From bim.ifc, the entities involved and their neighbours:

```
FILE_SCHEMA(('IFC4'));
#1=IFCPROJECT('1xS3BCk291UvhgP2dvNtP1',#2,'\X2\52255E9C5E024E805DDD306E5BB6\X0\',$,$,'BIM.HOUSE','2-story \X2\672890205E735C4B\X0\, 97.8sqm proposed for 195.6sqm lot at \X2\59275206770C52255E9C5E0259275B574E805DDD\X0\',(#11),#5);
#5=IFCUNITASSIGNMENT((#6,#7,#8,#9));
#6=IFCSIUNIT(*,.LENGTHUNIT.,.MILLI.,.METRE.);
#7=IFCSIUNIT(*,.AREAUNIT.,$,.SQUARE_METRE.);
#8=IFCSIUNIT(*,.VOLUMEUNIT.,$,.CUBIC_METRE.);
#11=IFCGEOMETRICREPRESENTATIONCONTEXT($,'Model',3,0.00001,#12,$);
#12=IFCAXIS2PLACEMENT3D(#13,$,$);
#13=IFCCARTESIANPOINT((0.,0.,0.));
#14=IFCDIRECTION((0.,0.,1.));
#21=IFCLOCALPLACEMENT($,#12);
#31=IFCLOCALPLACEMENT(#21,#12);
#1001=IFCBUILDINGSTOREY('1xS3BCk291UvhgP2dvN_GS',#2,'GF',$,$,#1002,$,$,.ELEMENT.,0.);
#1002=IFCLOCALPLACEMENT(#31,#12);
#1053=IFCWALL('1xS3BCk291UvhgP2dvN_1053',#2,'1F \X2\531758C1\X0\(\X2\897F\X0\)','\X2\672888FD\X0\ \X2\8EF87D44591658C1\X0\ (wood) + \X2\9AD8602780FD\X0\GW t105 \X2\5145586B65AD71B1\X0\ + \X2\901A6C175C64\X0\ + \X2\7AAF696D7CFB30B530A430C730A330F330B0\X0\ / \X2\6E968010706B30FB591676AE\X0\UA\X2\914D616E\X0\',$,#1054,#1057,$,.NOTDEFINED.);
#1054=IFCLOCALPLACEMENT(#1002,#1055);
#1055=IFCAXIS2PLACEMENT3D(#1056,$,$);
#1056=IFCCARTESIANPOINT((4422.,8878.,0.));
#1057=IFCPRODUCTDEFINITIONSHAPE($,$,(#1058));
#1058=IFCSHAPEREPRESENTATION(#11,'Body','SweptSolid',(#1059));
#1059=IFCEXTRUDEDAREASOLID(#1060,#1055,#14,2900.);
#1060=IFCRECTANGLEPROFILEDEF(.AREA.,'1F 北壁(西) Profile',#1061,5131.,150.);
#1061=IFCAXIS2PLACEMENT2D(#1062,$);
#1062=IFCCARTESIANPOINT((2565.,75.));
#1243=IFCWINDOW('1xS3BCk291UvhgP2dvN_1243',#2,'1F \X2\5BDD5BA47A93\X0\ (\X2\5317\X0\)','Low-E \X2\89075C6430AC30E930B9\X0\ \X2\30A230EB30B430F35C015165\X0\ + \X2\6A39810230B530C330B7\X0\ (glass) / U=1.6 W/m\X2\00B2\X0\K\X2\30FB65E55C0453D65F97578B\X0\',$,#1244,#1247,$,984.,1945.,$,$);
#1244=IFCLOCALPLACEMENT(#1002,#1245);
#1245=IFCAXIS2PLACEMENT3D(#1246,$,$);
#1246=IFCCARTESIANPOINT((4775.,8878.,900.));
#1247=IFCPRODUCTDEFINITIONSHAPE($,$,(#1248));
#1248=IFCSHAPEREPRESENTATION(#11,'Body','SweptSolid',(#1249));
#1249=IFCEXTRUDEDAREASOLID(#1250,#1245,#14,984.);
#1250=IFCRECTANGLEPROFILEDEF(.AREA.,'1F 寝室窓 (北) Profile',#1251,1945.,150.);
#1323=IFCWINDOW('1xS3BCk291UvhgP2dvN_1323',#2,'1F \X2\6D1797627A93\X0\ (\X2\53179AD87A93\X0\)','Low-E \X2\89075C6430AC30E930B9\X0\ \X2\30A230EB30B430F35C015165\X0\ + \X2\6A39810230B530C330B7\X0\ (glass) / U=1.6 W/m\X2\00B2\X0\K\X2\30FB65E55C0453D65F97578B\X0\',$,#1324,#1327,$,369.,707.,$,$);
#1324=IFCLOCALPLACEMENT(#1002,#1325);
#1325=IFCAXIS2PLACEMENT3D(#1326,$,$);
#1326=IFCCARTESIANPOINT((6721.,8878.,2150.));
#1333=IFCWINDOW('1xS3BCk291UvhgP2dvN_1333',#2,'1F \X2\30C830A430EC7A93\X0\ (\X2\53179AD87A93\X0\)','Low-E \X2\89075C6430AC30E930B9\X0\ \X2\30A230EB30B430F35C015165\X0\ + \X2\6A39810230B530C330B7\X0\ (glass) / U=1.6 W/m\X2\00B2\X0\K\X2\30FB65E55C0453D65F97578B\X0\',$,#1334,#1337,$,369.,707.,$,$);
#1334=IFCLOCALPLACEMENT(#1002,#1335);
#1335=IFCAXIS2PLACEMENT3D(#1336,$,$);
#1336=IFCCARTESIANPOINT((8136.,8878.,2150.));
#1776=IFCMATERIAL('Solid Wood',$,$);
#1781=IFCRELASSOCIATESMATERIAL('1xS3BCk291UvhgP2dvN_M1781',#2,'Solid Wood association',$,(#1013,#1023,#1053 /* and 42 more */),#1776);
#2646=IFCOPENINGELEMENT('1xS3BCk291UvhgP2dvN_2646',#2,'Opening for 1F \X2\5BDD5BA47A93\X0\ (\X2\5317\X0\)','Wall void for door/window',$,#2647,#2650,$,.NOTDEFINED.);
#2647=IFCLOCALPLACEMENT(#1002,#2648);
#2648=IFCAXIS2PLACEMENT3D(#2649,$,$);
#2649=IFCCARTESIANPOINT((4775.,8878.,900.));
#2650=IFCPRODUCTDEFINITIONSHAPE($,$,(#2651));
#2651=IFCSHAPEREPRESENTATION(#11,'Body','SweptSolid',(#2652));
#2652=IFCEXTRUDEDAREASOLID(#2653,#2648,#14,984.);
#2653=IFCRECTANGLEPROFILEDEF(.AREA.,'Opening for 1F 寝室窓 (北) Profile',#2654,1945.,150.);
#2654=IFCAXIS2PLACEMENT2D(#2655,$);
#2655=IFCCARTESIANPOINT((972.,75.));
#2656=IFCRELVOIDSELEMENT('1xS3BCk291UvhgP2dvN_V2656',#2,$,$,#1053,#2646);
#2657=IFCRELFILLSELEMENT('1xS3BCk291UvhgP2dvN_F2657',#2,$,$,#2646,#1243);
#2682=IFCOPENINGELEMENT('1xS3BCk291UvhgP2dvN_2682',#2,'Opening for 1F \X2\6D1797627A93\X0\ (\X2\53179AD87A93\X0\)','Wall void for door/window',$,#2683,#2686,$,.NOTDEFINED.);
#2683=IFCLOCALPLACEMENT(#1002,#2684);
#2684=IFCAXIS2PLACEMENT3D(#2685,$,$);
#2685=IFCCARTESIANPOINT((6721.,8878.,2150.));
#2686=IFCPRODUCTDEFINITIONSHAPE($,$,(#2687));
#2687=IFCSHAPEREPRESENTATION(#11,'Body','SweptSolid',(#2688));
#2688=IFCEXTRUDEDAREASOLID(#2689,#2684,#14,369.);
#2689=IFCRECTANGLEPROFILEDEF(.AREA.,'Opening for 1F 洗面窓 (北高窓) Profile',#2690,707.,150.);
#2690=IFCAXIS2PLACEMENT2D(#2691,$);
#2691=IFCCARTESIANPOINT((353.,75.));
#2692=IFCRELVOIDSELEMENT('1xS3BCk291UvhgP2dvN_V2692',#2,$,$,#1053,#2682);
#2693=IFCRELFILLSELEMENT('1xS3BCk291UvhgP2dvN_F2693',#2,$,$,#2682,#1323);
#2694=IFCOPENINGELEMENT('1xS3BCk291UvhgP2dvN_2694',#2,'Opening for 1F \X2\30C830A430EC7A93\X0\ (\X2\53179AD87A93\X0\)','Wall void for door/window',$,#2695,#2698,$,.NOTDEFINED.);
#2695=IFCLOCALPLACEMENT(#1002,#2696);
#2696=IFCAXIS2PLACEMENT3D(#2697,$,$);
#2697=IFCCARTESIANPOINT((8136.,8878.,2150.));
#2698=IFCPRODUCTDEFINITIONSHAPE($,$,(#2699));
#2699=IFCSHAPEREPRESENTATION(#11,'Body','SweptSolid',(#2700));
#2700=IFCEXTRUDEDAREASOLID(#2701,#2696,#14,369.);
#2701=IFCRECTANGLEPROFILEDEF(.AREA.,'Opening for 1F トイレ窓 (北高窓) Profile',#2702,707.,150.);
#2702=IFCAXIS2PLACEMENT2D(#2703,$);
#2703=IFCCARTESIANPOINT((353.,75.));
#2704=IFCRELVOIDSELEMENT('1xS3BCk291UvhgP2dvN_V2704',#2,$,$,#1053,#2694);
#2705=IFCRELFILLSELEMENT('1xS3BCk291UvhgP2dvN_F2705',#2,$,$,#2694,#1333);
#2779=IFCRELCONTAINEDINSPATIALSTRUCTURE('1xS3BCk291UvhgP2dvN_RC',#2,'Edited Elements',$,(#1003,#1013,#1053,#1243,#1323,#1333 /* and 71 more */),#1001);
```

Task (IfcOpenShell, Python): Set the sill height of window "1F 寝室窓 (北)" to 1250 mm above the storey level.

```python
import numpy as np
import ifcopenshell
import ifcopenshell.api.geometry
import ifcopenshell.geom
import ifcopenshell.util.element
import ifcopenshell.util.placement
import ifcopenshell.util.shape
import ifcopenshell.util.unit

model = ifcopenshell.open("bim.ifc")
unit_scale = ifcopenshell.util.unit.calculate_unit_scale(model)

window = model.by_guid("1xS3BCk291UvhgP2dvN_1243")
opening = window.FillsVoids[0].RelatingOpeningElement
storey = ifcopenshell.util.element.get_container(window, ifc_class="IfcBuildingStorey")
level = ifcopenshell.util.placement.get_local_placement(storey.ObjectPlacement)[2, 3]

# The opening's origin need not be at the sill, so measure its lowest point.
shape = ifcopenshell.geom.create_shape(ifcopenshell.geom.settings(), opening)
bottom = ifcopenshell.util.shape.get_shape_bottom_elevation(shape, shape.geometry) / unit_scale
dz = level + 1250.0 - bottom

shift = np.array([0.0, 0.0, dz])
# The window is not placed relative to its opening, so move both.
for product in (opening, window):
    matrix = ifcopenshell.util.placement.get_local_placement(product.ObjectPlacement)
    matrix[:3, 3] += shift
    ifcopenshell.api.geometry.edit_object_placement(model, product=product, matrix=matrix, is_si=False)

print(f"moved by {dz * unit_scale:+.3f} m")

model.write("bim-out.ifc")
```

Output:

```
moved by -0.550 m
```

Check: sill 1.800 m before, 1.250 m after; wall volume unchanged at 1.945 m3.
